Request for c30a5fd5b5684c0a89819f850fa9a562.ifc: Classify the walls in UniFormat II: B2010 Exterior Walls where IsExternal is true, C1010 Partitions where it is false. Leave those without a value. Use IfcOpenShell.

First a look at what the model holds.

```python
import ifcopenshell
import ifcopenshell.util.element

model = ifcopenshell.open("c30a5fd5b5684c0a89819f850fa9a562.ifc")
print(model.schema)
print("classifications:", [c.Name for c in model.by_type("IfcClassification")])
values = [ifcopenshell.util.element.get_pset(e, "Pset_WallCommon", "IsExternal") for e in model.by_type("IfcWall")]
for value in (True, False, None):
    print("IsExternal", value, values.count(value))
```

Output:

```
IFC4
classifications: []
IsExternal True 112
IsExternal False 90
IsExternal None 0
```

```python
import ifcopenshell
import ifcopenshell.api.classification
import ifcopenshell.util.element

model = ifcopenshell.open("c30a5fd5b5684c0a89819f850fa9a562.ifc")

system = ifcopenshell.api.classification.add_classification(model, classification="UniFormat II")

walls = model.by_type("IfcWall")
external = {e: ifcopenshell.util.element.get_pset(e, "Pset_WallCommon", "IsExternal") for e in walls}
for flag, code, name in ((True, "B2010", "Exterior Walls"), (False, "C1010", "Partitions")):
    products = [e for e in walls if external[e] is flag]
    ifcopenshell.api.classification.add_reference(
        model, products=products, classification=system, identification=code, name=name
    )
    print(code, len(products))

model.write("c30a5fd5b5684c0a89819f850fa9a562_v2.ifc")
```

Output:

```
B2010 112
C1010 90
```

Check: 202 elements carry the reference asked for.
